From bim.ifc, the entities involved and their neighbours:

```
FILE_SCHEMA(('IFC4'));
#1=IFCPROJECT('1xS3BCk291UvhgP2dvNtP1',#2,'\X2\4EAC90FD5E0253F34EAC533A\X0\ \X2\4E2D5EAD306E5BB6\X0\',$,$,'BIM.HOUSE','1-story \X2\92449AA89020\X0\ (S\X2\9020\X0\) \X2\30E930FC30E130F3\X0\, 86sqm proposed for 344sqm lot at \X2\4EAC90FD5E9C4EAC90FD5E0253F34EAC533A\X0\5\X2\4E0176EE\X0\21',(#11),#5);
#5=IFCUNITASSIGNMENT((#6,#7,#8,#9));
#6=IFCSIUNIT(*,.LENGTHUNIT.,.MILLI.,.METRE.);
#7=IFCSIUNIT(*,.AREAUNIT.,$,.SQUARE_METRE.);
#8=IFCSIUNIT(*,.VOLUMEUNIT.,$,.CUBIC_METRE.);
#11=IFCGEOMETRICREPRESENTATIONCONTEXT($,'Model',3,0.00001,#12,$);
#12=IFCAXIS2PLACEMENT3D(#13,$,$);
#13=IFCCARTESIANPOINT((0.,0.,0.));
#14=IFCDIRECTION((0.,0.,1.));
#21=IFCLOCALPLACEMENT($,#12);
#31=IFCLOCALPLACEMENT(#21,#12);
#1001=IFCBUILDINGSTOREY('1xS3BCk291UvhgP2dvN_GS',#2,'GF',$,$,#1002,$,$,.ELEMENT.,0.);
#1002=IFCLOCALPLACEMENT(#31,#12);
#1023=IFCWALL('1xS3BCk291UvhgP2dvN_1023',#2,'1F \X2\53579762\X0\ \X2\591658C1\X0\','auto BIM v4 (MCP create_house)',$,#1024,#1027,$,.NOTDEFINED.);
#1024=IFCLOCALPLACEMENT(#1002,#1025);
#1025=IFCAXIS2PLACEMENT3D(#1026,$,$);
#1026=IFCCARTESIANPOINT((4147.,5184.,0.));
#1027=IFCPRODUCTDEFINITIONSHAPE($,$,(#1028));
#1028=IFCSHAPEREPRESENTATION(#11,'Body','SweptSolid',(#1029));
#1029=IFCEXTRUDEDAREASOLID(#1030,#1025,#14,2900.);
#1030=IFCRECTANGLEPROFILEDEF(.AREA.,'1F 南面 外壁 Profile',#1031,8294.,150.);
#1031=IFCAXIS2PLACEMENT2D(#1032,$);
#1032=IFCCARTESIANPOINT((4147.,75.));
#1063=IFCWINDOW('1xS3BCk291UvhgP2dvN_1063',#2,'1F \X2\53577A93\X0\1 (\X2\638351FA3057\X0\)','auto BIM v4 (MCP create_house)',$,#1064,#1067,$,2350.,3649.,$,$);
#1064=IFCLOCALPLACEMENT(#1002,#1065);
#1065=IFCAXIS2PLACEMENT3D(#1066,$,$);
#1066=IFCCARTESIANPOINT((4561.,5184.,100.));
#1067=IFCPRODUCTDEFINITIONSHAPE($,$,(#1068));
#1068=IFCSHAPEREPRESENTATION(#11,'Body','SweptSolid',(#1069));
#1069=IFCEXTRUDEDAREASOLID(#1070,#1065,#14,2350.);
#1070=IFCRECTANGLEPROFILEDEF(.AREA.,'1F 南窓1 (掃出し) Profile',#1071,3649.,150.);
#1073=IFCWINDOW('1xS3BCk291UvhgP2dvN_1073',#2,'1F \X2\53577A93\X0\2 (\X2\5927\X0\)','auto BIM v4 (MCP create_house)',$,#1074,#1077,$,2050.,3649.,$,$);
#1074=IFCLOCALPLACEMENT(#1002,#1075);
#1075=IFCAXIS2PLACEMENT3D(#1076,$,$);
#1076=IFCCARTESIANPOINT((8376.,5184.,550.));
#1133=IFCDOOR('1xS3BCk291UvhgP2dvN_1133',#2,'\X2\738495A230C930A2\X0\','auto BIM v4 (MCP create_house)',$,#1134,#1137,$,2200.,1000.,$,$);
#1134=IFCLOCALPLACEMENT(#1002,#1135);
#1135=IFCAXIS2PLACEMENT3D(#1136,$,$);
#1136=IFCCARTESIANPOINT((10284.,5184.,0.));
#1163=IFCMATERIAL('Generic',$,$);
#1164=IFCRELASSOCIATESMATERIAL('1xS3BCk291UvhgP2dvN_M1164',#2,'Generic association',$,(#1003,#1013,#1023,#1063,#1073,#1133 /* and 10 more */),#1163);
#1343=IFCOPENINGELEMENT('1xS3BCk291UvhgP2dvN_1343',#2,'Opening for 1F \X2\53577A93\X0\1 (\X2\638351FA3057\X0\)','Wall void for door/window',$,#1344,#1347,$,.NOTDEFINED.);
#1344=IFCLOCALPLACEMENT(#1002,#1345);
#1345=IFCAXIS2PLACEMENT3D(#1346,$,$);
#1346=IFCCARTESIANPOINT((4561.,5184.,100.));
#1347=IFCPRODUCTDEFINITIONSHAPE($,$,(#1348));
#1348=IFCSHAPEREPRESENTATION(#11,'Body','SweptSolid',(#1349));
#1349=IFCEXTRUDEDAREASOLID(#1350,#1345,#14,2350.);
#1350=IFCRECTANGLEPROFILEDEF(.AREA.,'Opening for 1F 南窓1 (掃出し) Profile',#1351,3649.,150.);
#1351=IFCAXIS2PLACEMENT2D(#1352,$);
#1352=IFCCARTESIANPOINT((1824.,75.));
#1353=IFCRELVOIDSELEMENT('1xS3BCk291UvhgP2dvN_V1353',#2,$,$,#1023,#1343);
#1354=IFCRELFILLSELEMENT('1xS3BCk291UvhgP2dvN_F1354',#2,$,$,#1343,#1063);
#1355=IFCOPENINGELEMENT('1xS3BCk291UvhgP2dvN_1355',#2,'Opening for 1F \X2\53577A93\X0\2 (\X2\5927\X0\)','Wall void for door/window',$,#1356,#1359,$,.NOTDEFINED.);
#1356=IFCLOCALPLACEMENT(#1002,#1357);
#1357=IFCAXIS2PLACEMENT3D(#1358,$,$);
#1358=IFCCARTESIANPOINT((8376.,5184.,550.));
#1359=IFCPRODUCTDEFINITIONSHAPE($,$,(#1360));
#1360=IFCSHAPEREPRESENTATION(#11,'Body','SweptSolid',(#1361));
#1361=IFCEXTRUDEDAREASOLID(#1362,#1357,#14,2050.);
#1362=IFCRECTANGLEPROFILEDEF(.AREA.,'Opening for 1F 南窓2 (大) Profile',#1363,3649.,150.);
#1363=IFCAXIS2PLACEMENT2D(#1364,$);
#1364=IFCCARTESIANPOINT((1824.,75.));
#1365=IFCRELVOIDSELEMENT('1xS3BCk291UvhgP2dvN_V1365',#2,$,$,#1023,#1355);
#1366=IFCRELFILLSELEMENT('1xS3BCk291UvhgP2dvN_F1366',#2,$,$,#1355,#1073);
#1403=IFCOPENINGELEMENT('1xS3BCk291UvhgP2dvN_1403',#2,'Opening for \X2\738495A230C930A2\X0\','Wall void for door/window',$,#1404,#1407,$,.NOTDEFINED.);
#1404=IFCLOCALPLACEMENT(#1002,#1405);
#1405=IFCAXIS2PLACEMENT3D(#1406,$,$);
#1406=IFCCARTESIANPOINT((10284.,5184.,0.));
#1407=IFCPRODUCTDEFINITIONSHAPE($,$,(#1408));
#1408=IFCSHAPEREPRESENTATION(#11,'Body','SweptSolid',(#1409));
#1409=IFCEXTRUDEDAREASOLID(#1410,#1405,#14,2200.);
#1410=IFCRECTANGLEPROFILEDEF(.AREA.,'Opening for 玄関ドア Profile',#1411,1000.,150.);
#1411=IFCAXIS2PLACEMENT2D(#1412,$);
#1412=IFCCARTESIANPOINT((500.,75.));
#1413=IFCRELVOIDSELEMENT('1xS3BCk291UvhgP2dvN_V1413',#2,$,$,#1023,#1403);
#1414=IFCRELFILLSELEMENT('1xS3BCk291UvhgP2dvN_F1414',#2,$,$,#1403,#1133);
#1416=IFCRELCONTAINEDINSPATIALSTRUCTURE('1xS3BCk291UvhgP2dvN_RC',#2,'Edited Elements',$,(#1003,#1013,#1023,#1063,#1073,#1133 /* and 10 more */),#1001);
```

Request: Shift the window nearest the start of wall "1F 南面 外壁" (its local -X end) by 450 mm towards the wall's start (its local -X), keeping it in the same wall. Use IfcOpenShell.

```python
import ifcopenshell
import ifcopenshell.api.geometry
import ifcopenshell.util.placement

model = ifcopenshell.open("bim.ifc")

window = model.by_guid("1xS3BCk291UvhgP2dvN_1063")
opening = window.FillsVoids[0].RelatingOpeningElement
wall = opening.VoidsElements[0].RelatingBuildingElement

wall_matrix = ifcopenshell.util.placement.get_local_placement(wall.ObjectPlacement)
shift = wall_matrix[:3, 0] * -450.0
before = ifcopenshell.util.placement.get_local_placement(window.ObjectPlacement)[:3, 3].copy()

# The window is not placed relative to its opening, so move both.
for product in (opening, window):
    matrix = ifcopenshell.util.placement.get_local_placement(product.ObjectPlacement)
    matrix[:3, 3] += shift
    ifcopenshell.api.geometry.edit_object_placement(model, product=product, matrix=matrix, is_si=False)

after = ifcopenshell.util.placement.get_local_placement(window.ObjectPlacement)[:3, 3]
print("window moved by", (after - before).round(3) + 0.0)

model.write("bim_rev.ifc")
```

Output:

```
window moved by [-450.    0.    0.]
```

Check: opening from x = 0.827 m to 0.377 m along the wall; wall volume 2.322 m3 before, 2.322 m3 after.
